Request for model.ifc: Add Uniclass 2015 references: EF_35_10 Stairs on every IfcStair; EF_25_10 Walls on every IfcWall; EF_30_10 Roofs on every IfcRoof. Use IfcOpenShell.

First a look at what the model holds.

```python
import ifcopenshell

model = ifcopenshell.open("model.ifc")
print(model.schema)
print("classifications:", [c.Name for c in model.by_type("IfcClassification")])
for ifc_class in ("IfcDoor", "IfcRoof", "IfcStair", "IfcWall", "IfcWindow"):
    print(ifc_class, len(model.by_type(ifc_class)))
```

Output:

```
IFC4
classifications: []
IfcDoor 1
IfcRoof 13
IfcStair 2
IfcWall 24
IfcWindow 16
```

```python
import ifcopenshell
import ifcopenshell.api.classification

model = ifcopenshell.open("model.ifc")

system = ifcopenshell.api.classification.add_classification(model, classification="Uniclass 2015")

codes = {
    "IfcStair": ("EF_35_10", "Stairs"),
    "IfcWall": ("EF_25_10", "Walls"),
    "IfcRoof": ("EF_30_10", "Roofs"),
}
for ifc_class, (code, name) in codes.items():
    products = model.by_type(ifc_class)
    ifcopenshell.api.classification.add_reference(
        model, products=products, classification=system, identification=code, name=name
    )
    print(code, len(products))

model.write("model-out.ifc")
```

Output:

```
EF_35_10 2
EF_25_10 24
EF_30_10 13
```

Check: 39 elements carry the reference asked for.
